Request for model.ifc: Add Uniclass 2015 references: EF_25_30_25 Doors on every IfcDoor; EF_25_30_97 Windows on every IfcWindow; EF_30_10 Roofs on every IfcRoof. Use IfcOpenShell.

First a look at what the model holds.

```python
import ifcopenshell

model = ifcopenshell.open("model.ifc")
print(model.schema)
print("classifications:", [c.Name for c in model.by_type("IfcClassification")])
for ifc_class in ("IfcDoor", "IfcRoof", "IfcStair", "IfcWall", "IfcWindow"):
    print(ifc_class, len(model.by_type(ifc_class)))
```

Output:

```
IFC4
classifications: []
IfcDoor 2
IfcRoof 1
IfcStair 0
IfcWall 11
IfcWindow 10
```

```python
import ifcopenshell
import ifcopenshell.api.classification

model = ifcopenshell.open("model.ifc")

system = ifcopenshell.api.classification.add_classification(model, classification="Uniclass 2015")

codes = {
    "IfcDoor": ("EF_25_30_25", "Doors"),
    "IfcWindow": ("EF_25_30_97", "Windows"),
    "IfcRoof": ("EF_30_10", "Roofs"),
}
for ifc_class, (code, name) in codes.items():
    products = model.by_type(ifc_class)
    ifcopenshell.api.classification.add_reference(
        model, products=products, classification=system, identification=code, name=name
    )
    print(code, len(products))

model.write("model_edited.ifc")
```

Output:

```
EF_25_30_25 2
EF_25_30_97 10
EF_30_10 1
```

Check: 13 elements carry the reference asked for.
